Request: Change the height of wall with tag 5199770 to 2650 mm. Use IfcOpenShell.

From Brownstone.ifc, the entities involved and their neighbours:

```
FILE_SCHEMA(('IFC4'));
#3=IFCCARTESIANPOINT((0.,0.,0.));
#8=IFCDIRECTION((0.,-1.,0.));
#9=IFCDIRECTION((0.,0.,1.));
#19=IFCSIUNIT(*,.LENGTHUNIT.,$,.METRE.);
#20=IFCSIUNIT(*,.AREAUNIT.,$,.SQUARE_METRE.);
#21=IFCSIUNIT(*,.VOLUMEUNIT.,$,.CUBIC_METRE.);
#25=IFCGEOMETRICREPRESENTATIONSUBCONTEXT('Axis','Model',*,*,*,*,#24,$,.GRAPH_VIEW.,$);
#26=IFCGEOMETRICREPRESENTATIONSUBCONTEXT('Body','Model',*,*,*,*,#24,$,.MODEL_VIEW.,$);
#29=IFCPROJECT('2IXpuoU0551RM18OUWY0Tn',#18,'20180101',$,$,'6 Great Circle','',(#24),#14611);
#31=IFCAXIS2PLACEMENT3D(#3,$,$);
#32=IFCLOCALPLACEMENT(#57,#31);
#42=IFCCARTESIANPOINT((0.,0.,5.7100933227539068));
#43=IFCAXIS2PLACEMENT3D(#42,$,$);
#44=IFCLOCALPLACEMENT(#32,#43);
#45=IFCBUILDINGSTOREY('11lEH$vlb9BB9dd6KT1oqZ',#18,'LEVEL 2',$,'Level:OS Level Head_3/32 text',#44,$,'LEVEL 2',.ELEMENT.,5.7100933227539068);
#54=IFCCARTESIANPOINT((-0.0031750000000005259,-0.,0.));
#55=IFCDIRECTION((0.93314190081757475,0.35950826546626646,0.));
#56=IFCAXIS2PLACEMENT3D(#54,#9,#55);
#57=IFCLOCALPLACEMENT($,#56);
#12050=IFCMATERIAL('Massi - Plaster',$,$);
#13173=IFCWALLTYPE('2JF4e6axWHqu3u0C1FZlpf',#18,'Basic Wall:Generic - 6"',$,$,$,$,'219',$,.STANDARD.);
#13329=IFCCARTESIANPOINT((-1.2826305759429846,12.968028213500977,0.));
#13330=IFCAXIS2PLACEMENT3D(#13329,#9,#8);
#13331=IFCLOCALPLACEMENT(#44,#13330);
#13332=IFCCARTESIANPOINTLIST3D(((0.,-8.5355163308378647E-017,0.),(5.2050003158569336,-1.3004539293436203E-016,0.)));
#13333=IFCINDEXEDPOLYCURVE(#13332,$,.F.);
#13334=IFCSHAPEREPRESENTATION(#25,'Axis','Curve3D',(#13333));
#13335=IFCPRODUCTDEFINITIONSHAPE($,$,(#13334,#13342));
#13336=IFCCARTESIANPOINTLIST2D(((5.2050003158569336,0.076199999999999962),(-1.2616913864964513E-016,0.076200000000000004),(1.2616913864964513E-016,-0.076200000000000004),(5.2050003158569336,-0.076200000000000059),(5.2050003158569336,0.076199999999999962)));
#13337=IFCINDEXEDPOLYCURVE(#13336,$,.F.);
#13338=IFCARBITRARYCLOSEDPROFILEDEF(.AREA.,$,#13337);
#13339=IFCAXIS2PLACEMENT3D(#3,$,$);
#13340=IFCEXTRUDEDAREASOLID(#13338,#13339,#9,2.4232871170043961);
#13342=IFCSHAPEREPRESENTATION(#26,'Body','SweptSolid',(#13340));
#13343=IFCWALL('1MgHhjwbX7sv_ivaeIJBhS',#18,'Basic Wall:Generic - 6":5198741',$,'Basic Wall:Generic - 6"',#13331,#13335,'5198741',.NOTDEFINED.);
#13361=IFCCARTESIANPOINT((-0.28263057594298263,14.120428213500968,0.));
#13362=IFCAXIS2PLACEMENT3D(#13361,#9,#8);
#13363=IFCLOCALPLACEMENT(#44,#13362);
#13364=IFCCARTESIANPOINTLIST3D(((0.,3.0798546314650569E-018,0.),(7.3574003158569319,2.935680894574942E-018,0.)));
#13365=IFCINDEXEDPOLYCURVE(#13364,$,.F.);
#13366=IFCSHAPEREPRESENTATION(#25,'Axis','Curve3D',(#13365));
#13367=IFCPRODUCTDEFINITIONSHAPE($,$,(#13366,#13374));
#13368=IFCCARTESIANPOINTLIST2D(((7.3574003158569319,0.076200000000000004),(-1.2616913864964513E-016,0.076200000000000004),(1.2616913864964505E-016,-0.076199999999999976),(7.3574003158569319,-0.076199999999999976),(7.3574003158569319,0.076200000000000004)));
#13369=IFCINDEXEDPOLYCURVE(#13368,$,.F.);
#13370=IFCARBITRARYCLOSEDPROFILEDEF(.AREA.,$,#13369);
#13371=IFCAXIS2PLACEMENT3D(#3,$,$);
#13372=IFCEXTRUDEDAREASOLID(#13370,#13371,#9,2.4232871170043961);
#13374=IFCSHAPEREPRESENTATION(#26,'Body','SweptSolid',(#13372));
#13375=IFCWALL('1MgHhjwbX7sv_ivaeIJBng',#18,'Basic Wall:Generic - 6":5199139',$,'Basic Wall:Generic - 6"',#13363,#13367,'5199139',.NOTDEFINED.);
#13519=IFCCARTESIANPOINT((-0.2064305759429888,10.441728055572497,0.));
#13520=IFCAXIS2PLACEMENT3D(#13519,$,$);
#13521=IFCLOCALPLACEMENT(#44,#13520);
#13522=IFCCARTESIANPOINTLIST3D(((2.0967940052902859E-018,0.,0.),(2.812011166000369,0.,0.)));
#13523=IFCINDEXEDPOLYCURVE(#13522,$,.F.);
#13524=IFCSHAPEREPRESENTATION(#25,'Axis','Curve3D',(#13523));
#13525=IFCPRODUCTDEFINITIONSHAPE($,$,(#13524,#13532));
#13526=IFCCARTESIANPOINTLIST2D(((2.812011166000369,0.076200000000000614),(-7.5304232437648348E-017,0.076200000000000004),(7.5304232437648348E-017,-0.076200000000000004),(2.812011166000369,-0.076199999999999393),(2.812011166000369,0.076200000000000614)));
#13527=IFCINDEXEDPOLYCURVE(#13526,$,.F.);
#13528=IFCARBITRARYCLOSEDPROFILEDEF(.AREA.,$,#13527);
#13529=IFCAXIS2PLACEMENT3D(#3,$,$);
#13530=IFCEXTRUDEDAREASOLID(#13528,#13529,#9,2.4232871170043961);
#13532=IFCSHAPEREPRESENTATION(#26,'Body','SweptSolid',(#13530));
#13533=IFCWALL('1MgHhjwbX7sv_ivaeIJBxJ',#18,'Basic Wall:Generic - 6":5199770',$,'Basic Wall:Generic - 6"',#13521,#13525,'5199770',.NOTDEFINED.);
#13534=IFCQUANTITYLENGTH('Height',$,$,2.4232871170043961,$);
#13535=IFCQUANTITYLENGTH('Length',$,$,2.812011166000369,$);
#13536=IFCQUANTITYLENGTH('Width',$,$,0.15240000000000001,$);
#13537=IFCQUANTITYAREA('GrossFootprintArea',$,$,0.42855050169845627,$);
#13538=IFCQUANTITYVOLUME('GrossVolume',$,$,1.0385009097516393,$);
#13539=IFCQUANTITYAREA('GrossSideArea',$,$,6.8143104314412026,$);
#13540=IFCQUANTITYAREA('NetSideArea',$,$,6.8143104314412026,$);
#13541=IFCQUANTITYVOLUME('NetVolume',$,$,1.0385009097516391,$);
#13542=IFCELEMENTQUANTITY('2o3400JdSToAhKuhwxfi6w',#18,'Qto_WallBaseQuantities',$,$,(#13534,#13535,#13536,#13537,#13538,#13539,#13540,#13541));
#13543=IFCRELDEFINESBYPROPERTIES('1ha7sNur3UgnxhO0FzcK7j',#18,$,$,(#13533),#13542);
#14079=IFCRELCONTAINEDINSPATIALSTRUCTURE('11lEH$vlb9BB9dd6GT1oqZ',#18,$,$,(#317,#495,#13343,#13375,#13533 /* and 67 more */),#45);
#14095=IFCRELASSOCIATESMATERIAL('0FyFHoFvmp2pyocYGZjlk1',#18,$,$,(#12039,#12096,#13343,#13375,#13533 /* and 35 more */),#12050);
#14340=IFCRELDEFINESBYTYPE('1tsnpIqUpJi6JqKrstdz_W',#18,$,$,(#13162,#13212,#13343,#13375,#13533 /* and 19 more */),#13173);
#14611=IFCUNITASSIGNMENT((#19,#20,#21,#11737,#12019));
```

```python
import ifcopenshell
import ifcopenshell.api.pset
import ifcopenshell.geom
import ifcopenshell.util.element
import ifcopenshell.util.representation
import ifcopenshell.util.shape
import ifcopenshell.util.unit

model = ifcopenshell.open("Brownstone.ifc")
unit_scale = ifcopenshell.util.unit.calculate_unit_scale(model)
area_scale = ifcopenshell.util.unit.calculate_unit_scale(model, "AREAUNIT")
volume_scale = ifcopenshell.util.unit.calculate_unit_scale(model, "VOLUMEUNIT")
settings = ifcopenshell.geom.settings()


def volume(element):
    """Net volume in cubic metres, openings subtracted."""
    shape = ifcopenshell.geom.create_shape(settings, element)
    return ifcopenshell.util.shape.get_volume(shape.geometry)


wall = model.by_guid("1MgHhjwbX7sv_ivaeIJBxJ")
before = volume(wall)

body = ifcopenshell.util.representation.get_representation(wall, "Model", "Body")
solid = body.Items[0]
old_height = solid.Depth
solid.Depth = 2.65
after = volume(wall)
thickness = 0.1524  # wall thickness in metres

# Update the stored height, areas and volumes.
qto = model.by_id(ifcopenshell.util.element.get_pset(wall, "Qto_WallBaseQuantities", should_inherit=False)["id"])
ifcopenshell.api.pset.edit_qto(model, qto=qto, properties={
    "Height": solid.Depth,
    "GrossVolume": ifcopenshell.util.element.get_pset(wall, "Qto_WallBaseQuantities", "GrossVolume") * solid.Depth / old_height,
    "GrossSideArea": ifcopenshell.util.element.get_pset(wall, "Qto_WallBaseQuantities", "GrossSideArea") * solid.Depth / old_height,
    "NetSideArea": after / thickness / area_scale,
    "NetVolume": after / volume_scale,
})

print(f"height {old_height:g} -> {solid.Depth:g}, volume {before:.3f} -> {after:.3f} m3")

model.write("Brownstone_v2.ifc")
```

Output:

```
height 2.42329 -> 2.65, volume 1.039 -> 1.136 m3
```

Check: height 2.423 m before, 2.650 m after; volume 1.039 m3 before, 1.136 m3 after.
